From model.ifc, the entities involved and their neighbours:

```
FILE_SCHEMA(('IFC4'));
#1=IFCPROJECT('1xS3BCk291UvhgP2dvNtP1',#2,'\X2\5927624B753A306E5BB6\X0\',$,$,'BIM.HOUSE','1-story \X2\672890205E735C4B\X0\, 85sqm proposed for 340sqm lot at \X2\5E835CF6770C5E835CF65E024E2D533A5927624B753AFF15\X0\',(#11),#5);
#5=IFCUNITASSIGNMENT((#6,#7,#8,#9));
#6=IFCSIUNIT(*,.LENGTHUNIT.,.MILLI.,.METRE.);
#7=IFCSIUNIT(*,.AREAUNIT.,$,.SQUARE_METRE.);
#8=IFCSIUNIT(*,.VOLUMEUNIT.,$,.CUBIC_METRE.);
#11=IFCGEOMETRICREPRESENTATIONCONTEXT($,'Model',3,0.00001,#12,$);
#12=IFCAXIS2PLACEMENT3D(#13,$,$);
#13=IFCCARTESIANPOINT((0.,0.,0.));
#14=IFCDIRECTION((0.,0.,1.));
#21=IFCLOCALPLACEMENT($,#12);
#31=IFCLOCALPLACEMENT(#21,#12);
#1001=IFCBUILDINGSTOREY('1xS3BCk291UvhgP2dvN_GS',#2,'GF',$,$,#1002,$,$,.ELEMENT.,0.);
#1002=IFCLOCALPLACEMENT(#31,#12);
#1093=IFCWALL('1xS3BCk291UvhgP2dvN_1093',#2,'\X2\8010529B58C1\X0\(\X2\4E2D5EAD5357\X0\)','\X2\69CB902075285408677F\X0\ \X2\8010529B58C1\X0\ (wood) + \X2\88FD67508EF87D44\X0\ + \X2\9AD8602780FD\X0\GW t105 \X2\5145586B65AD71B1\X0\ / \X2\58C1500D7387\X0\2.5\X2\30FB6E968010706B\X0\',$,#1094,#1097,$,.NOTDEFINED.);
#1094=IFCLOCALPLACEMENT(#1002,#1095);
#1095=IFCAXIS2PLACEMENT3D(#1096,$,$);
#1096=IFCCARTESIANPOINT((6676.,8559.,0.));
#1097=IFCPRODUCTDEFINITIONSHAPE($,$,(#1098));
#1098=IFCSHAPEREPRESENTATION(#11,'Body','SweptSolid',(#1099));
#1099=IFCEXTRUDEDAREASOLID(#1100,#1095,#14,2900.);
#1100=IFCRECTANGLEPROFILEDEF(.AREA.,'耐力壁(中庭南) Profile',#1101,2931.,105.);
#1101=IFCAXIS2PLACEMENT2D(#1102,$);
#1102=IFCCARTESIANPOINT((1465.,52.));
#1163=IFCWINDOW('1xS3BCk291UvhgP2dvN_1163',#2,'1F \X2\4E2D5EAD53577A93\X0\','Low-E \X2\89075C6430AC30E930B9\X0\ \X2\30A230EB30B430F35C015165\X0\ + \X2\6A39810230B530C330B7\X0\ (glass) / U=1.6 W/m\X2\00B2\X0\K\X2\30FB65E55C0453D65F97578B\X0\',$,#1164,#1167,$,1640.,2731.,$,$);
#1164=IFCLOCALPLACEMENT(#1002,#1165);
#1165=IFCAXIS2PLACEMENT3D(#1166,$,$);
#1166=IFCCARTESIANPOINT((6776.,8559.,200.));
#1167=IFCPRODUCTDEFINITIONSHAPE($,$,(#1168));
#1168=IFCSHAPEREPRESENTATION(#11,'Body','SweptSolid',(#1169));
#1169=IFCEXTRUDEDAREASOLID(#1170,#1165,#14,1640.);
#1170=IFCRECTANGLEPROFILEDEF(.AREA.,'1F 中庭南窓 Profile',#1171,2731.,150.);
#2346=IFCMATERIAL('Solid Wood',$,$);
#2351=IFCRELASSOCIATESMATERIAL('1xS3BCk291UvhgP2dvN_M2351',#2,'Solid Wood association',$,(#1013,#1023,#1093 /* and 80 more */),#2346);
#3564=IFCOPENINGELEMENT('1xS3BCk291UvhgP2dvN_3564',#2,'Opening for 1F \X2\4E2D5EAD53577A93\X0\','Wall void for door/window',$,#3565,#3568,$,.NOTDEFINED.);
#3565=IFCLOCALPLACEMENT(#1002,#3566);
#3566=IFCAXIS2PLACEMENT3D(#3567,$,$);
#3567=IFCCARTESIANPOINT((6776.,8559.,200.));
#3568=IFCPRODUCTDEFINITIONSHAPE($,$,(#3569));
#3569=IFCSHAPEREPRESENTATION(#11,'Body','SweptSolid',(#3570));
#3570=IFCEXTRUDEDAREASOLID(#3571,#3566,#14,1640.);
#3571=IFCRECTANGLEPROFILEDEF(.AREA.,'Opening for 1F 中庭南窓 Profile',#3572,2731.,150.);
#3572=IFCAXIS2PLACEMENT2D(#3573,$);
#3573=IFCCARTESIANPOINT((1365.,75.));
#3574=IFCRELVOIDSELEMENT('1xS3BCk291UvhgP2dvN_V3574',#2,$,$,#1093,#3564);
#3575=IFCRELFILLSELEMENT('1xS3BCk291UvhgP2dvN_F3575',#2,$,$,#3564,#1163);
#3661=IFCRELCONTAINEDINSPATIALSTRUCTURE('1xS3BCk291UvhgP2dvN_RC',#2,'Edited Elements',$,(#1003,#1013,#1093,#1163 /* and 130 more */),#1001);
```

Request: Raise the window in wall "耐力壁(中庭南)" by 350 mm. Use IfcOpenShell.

```python
import numpy as np
import ifcopenshell
import ifcopenshell.api.geometry
import ifcopenshell.util.placement
import ifcopenshell.util.unit

model = ifcopenshell.open("model.ifc")
unit_scale = ifcopenshell.util.unit.calculate_unit_scale(model)

window = model.by_guid("1xS3BCk291UvhgP2dvN_1163")
opening = window.FillsVoids[0].RelatingOpeningElement
dz = 350.0

shift = np.array([0.0, 0.0, dz])
# The window is not placed relative to its opening, so move both.
for product in (opening, window):
    matrix = ifcopenshell.util.placement.get_local_placement(product.ObjectPlacement)
    matrix[:3, 3] += shift
    ifcopenshell.api.geometry.edit_object_placement(model, product=product, matrix=matrix, is_si=False)

print(f"moved by {dz * unit_scale:+.3f} m")

model.write("model_rev.ifc")
```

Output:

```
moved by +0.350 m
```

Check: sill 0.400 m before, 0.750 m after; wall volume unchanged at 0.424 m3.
